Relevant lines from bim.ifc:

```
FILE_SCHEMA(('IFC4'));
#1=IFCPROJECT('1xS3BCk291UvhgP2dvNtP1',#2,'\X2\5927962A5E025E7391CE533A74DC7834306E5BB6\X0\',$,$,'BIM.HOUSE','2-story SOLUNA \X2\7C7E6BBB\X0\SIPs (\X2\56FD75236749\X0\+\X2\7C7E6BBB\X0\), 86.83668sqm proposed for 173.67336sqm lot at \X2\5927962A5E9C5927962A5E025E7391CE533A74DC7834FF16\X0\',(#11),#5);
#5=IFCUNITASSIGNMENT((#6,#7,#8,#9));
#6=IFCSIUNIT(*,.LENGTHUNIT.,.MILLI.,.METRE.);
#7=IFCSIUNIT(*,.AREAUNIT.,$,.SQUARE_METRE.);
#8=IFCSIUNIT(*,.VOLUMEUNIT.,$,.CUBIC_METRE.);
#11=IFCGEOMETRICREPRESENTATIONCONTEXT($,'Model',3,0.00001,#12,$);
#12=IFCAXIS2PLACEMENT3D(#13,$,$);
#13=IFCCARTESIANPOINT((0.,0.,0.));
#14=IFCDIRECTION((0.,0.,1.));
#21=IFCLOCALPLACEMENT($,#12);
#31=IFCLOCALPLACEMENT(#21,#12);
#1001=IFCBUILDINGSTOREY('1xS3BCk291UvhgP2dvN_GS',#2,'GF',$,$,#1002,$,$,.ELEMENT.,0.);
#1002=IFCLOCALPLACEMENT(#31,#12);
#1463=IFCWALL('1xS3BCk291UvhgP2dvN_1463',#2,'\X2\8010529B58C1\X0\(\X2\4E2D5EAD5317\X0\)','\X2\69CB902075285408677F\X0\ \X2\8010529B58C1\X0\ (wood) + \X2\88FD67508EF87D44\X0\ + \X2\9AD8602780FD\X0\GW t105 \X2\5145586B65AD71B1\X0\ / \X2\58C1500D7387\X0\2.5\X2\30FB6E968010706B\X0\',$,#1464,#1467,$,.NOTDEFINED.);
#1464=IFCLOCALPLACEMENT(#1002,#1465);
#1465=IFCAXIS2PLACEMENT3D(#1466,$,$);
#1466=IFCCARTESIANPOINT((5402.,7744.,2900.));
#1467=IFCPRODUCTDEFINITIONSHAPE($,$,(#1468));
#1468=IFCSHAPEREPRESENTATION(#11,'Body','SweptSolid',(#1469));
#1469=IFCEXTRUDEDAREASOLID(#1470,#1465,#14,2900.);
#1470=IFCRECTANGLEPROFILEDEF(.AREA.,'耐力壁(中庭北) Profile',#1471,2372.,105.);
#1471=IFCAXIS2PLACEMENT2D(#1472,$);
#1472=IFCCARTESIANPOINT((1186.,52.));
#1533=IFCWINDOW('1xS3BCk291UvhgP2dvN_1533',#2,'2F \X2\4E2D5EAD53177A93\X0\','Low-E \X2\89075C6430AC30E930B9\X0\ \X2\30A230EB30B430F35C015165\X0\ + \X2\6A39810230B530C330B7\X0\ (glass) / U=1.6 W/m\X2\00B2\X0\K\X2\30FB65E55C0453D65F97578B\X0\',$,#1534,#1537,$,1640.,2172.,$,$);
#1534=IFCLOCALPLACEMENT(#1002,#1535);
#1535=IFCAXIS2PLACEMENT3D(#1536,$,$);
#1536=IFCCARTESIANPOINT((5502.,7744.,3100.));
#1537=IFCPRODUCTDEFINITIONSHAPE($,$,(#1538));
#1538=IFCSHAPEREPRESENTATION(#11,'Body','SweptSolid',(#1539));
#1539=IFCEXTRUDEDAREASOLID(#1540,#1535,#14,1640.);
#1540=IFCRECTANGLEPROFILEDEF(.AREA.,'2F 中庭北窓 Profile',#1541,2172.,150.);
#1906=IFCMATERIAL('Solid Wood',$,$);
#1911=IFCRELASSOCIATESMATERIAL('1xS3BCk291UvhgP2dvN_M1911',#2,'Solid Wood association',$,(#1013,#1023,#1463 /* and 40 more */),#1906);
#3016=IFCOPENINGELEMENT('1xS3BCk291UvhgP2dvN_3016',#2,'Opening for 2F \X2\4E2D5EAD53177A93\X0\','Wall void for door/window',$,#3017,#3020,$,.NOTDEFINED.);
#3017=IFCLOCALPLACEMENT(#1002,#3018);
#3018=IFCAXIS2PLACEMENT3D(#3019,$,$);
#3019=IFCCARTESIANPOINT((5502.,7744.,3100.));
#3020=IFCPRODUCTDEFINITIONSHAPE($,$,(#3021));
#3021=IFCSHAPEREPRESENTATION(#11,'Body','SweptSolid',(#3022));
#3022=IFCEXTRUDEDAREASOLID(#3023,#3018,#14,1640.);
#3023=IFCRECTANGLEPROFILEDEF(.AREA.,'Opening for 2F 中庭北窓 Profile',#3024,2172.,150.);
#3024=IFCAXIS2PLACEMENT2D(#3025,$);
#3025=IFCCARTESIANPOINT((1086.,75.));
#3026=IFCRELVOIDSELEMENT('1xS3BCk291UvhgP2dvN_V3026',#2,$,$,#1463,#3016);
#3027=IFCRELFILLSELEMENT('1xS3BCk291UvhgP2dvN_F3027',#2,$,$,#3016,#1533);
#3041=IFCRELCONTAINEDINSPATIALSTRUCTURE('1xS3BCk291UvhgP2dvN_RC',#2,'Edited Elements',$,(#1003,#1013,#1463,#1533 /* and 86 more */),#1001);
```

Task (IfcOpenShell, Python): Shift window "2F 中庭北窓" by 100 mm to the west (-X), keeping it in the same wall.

```python
import ifcopenshell
import ifcopenshell.api.geometry
import ifcopenshell.util.placement
import ifcopenshell.util.unit

model = ifcopenshell.open("bim.ifc")
unit_scale = ifcopenshell.util.unit.calculate_unit_scale(model)

window = model.by_guid("1xS3BCk291UvhgP2dvN_1533")
opening = window.FillsVoids[0].RelatingOpeningElement
wall = opening.VoidsElements[0].RelatingBuildingElement

wall_matrix = ifcopenshell.util.placement.get_local_placement(wall.ObjectPlacement)
shift = wall_matrix[:3, 0] * -0.1 / unit_scale
before = ifcopenshell.util.placement.get_local_placement(window.ObjectPlacement)[:3, 3].copy()

# The window is not placed relative to its opening, so move both.
for product in (opening, window):
    matrix = ifcopenshell.util.placement.get_local_placement(product.ObjectPlacement)
    matrix[:3, 3] += shift
    ifcopenshell.api.geometry.edit_object_placement(model, product=product, matrix=matrix, is_si=False)

after = ifcopenshell.util.placement.get_local_placement(window.ObjectPlacement)[:3, 3]
print("window moved by", (after - before).round(3) + 0.0)

model.write("bim-out.ifc")
```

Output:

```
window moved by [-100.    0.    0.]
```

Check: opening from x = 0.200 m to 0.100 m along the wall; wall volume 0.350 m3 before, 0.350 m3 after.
